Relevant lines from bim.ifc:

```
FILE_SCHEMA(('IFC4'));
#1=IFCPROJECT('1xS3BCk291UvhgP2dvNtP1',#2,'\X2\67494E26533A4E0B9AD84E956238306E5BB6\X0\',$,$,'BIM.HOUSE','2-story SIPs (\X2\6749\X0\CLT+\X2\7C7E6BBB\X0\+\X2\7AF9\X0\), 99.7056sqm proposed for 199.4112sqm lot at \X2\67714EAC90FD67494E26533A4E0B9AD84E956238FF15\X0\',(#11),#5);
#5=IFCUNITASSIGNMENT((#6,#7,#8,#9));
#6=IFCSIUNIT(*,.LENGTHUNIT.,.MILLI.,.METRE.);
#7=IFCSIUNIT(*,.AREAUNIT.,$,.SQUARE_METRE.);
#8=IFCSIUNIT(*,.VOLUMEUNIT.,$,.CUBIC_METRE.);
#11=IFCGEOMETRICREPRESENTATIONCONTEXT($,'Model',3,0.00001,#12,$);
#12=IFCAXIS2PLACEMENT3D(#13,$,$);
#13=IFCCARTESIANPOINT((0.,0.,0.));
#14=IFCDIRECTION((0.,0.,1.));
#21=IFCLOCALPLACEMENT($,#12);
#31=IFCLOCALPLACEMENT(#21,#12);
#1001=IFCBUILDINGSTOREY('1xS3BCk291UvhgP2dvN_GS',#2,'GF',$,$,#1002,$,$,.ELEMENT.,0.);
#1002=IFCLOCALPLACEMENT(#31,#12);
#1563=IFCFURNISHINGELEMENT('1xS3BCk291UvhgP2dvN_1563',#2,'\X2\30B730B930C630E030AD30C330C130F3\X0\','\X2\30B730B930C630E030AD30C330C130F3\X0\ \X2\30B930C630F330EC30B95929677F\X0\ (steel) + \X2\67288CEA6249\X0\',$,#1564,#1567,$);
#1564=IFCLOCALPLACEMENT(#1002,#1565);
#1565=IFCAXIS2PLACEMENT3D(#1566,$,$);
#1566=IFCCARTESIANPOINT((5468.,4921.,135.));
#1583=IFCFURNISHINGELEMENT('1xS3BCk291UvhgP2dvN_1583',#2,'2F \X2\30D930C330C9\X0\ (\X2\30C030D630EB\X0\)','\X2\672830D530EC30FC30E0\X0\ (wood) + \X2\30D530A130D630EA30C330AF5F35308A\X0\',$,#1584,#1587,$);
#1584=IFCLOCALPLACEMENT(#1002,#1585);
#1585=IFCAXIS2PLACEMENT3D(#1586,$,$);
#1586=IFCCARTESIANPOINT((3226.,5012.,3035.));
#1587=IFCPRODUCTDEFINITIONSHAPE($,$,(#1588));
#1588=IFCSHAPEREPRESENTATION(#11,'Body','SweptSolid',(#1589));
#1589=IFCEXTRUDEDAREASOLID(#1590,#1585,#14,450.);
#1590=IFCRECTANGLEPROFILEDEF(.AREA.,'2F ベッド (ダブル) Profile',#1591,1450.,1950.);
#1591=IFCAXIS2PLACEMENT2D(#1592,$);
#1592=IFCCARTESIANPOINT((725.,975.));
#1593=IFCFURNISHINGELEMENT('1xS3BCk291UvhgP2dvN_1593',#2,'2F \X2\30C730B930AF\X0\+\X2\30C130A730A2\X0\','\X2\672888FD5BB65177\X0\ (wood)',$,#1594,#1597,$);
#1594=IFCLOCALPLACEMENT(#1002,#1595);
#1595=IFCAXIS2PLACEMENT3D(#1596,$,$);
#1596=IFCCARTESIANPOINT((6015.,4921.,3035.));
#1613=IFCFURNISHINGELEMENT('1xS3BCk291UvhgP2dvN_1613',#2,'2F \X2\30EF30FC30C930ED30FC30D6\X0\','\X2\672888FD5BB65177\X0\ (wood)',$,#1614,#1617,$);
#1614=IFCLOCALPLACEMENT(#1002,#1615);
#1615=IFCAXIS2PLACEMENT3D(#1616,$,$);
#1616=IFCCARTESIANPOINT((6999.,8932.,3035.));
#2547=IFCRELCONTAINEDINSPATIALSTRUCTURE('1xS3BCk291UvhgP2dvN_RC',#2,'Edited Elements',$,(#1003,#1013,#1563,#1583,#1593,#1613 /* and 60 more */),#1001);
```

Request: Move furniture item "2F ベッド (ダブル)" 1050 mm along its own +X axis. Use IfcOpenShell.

```python
import ifcopenshell
import ifcopenshell.api.geometry
import ifcopenshell.util.placement

model = ifcopenshell.open("bim.ifc")

item = model.by_guid("1xS3BCk291UvhgP2dvN_1583")
matrix = ifcopenshell.util.placement.get_local_placement(item.ObjectPlacement)
matrix[:3, 3] += matrix[:3, 0] * 1050.0
ifcopenshell.api.geometry.edit_object_placement(model, product=item, matrix=matrix, is_si=False)

print(ifcopenshell.util.placement.get_local_placement(item.ObjectPlacement).round(3) + 0.0)

model.write("bim_updated.ifc")
```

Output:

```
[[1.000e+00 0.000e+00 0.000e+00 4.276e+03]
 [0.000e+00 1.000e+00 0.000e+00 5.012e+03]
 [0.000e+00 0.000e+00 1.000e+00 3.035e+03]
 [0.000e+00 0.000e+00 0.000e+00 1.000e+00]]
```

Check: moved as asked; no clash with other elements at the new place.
